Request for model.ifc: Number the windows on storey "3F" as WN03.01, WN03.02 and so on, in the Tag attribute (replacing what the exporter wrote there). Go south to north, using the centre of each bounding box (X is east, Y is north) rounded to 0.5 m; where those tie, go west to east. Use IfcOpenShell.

First a look at what the model holds.

```python
import ifcopenshell
import ifcopenshell.util.element
import ifcopenshell.util.placement

model = ifcopenshell.open("model.ifc")
print(model.schema)
storey = next(s for s in model.by_type("IfcBuildingStorey") if s.Name == "3F")
windows = [e for e in ifcopenshell.util.element.get_decomposition(storey) if e.is_a("IfcWindow")]
for e in sorted(windows, key=lambda e: e.id()):
    origin = ifcopenshell.util.placement.get_local_placement(e.ObjectPlacement)[:3, 3]
    print(e.id(), e.Tag, e.Name, origin.round(2) + 0.0, sep=" | ")
```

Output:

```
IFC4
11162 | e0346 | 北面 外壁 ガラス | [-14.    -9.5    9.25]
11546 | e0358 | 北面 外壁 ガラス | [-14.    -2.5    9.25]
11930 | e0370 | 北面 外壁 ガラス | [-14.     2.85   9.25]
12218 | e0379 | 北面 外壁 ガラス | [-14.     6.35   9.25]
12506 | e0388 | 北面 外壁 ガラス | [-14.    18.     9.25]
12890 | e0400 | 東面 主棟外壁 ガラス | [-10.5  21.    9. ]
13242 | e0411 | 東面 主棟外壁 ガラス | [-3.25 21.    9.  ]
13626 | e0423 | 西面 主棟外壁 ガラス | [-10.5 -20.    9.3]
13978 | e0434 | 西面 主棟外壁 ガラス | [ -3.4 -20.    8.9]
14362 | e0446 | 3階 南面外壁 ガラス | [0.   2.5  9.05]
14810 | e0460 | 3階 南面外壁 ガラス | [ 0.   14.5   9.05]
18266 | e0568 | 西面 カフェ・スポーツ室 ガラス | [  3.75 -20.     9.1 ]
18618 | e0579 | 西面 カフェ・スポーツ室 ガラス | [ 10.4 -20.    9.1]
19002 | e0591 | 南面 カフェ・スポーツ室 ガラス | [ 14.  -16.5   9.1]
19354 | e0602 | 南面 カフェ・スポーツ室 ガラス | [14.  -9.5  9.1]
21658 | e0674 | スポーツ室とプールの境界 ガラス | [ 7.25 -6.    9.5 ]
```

```python
import ifcopenshell
import ifcopenshell.geom
import ifcopenshell.util.element
import ifcopenshell.util.shape

model = ifcopenshell.open("model.ifc")
settings = ifcopenshell.geom.settings()
settings.set("use-world-coords", True)


def centre(element):
    shape = ifcopenshell.geom.create_shape(settings, element)
    return ifcopenshell.util.shape.get_bbox_centroid(shape.geometry)


storey = next(s for s in model.by_type("IfcBuildingStorey") if s.Name == "3F")
windows = [e for e in ifcopenshell.util.element.get_decomposition(storey) if e.is_a("IfcWindow")]

# Insertion points can sit at a corner or the storey origin, so sort by the geometry (in metres).
centres = {e: centre(e) for e in windows}
windows.sort(key=lambda e: (round(centres[e][1] / 0.5), centres[e][0]))

for i, e in enumerate(windows, start=1):
    number = f"WN03.{i:02d}"
    e.Tag = number
    print(e.id(), number)

model.write("model_rev.ifc")
```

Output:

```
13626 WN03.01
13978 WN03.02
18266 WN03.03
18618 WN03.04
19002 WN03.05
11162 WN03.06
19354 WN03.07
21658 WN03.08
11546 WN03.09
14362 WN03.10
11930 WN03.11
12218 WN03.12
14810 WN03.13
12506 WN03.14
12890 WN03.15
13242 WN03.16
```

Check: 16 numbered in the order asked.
